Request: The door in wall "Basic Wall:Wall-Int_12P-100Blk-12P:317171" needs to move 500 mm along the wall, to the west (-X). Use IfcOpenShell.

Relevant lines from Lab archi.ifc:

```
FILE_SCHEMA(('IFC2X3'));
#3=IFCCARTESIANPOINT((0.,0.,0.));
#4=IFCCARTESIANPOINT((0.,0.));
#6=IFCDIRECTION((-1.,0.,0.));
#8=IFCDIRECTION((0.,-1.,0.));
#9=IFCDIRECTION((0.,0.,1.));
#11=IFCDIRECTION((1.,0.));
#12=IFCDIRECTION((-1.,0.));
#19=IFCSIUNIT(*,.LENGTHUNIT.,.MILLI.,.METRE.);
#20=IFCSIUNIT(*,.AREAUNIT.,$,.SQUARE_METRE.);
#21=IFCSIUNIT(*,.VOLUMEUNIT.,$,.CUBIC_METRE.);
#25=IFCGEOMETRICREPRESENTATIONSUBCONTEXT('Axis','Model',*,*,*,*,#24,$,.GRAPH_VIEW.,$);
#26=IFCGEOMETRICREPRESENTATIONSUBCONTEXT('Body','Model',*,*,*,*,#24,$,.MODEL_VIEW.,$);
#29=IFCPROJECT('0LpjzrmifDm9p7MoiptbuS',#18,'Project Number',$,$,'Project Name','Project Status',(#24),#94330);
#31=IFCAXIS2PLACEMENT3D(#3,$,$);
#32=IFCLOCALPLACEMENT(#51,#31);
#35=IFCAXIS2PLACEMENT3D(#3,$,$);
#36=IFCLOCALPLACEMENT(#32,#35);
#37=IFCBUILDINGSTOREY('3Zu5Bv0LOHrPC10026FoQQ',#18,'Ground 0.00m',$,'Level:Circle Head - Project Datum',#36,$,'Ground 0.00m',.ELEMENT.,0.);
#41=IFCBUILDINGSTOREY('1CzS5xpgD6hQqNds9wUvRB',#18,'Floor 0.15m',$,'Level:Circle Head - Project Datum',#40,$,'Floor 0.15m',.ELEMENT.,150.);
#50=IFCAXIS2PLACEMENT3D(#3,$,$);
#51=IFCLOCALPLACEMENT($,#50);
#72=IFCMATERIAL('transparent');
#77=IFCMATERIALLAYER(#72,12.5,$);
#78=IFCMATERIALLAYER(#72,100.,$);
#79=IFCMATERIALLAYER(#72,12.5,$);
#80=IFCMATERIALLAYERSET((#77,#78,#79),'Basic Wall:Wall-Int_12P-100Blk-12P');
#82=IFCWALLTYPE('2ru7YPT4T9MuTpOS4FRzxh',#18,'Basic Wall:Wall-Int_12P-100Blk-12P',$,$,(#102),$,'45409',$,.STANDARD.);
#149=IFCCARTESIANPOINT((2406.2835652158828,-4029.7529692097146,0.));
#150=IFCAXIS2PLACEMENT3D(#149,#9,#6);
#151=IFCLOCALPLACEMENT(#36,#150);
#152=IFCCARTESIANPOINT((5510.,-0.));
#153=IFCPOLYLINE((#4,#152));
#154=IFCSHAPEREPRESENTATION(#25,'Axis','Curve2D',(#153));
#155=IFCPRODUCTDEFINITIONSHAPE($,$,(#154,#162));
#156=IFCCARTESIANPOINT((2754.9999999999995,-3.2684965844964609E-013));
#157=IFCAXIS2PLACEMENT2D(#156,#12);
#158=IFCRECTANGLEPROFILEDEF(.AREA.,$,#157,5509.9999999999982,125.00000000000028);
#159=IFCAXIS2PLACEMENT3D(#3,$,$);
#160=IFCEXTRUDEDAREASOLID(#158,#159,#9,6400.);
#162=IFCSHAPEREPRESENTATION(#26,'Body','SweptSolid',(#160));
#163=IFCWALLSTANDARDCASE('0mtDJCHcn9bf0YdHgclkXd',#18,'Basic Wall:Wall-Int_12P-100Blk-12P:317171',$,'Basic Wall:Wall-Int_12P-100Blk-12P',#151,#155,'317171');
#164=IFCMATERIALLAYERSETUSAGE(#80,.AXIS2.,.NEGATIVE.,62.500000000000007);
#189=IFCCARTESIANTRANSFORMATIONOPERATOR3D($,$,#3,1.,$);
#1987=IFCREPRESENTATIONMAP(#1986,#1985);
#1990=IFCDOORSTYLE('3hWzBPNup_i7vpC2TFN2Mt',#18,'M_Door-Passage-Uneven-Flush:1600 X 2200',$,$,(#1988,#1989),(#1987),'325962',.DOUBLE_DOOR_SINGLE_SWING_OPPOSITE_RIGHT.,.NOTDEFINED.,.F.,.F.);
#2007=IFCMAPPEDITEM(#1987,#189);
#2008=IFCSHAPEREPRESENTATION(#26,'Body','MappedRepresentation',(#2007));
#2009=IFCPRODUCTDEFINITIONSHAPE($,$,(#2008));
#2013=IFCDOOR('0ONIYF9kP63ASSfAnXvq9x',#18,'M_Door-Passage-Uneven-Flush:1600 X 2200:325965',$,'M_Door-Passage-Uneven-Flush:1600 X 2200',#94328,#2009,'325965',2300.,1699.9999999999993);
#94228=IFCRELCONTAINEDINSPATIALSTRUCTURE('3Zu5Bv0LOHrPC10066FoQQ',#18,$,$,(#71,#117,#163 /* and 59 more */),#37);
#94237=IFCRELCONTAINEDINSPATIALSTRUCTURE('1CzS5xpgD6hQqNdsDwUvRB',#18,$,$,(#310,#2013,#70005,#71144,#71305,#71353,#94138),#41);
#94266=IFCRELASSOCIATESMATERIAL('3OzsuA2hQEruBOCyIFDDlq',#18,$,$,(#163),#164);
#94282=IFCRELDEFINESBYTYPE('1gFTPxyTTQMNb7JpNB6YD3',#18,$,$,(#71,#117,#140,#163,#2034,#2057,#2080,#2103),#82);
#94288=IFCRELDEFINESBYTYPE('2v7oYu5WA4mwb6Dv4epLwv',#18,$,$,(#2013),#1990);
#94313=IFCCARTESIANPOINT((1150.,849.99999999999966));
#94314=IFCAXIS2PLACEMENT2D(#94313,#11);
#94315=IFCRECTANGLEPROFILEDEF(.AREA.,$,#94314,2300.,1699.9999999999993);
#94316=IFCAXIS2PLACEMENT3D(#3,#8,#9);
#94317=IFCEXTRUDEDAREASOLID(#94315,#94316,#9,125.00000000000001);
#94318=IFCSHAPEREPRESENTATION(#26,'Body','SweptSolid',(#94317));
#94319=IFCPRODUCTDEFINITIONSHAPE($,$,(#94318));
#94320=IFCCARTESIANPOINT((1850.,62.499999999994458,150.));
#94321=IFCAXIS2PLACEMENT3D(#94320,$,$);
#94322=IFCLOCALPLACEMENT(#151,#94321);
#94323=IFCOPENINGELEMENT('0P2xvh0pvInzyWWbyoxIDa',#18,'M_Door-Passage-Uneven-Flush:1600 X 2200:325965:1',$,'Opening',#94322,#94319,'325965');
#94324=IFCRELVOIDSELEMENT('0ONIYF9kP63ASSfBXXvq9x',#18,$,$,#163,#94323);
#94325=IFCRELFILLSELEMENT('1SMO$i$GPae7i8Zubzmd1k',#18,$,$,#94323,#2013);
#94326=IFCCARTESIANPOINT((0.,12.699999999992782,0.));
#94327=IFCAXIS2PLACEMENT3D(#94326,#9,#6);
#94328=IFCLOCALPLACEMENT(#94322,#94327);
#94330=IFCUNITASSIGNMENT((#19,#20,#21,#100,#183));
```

```python
import ifcopenshell
import ifcopenshell.api.geometry
import ifcopenshell.util.placement
import ifcopenshell.util.unit

model = ifcopenshell.open("Lab archi.ifc")
unit_scale = ifcopenshell.util.unit.calculate_unit_scale(model)

door = model.by_id(2013)
opening = door.FillsVoids[0].RelatingOpeningElement
wall = opening.VoidsElements[0].RelatingBuildingElement

wall_matrix = ifcopenshell.util.placement.get_local_placement(wall.ObjectPlacement)
shift = wall_matrix[:3, 0] * 0.5 / unit_scale
before = ifcopenshell.util.placement.get_local_placement(door.ObjectPlacement)[:3, 3].copy()

# The door is placed relative to its opening, so it follows when the opening moves.
matrix = ifcopenshell.util.placement.get_local_placement(opening.ObjectPlacement)
matrix[:3, 3] += shift
ifcopenshell.api.geometry.edit_object_placement(
    model, product=opening, matrix=matrix, is_si=False, should_transform_children=True
)

after = ifcopenshell.util.placement.get_local_placement(door.ObjectPlacement)[:3, 3]
print("door moved by", (after - before).round(3) + 0.0)

model.write("Lab archi_edited.ifc")
```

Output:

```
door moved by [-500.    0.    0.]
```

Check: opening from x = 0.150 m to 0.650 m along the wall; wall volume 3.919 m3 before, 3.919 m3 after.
